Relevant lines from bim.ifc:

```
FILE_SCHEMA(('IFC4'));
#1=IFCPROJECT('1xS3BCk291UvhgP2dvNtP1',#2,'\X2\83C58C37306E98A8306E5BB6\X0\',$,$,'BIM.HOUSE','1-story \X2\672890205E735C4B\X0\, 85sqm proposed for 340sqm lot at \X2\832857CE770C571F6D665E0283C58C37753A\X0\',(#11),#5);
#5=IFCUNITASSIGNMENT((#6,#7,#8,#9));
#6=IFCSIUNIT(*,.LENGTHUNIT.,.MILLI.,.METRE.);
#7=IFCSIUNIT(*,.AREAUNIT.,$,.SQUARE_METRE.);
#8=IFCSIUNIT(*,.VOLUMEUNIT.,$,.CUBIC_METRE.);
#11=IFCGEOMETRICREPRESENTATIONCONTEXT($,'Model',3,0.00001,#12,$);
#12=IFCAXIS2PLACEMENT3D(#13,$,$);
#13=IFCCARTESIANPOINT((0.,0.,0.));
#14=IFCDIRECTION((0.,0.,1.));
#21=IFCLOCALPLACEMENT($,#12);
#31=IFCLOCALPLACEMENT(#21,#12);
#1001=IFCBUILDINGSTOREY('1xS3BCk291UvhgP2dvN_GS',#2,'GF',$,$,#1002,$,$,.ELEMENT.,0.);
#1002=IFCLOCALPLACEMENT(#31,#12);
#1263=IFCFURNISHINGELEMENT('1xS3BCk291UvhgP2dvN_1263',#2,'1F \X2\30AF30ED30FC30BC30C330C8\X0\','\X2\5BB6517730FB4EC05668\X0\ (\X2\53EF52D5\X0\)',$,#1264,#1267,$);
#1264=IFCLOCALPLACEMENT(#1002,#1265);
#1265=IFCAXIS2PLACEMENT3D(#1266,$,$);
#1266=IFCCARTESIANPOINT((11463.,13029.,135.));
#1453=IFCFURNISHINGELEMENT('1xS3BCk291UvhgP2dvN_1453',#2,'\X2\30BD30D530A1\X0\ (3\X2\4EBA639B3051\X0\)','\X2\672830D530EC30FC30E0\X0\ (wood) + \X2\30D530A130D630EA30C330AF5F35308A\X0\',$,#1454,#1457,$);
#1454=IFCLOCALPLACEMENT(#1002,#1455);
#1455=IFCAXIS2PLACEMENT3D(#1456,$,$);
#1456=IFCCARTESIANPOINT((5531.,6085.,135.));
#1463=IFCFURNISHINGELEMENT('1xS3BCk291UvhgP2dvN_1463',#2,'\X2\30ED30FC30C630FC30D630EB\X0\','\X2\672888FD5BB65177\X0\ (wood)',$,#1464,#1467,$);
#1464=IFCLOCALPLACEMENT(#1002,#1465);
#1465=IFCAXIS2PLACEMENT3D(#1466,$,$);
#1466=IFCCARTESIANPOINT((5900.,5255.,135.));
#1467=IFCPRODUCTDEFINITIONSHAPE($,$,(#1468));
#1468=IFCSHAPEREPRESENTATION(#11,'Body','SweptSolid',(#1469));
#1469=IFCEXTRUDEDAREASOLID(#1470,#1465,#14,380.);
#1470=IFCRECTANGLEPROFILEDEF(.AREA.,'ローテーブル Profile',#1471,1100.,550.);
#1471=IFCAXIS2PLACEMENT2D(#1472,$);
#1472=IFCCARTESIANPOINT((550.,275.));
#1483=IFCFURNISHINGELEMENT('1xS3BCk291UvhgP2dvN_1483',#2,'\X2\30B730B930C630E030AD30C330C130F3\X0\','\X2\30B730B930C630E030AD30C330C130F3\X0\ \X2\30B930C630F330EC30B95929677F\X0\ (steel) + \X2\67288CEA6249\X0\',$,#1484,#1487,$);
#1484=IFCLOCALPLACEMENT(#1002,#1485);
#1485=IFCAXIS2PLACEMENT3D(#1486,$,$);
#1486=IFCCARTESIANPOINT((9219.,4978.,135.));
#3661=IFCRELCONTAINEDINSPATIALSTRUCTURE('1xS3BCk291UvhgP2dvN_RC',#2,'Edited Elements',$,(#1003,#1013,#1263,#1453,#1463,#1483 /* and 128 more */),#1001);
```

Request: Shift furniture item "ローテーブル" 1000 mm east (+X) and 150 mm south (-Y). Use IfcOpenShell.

```python
import ifcopenshell
import ifcopenshell.api.geometry
import ifcopenshell.util.placement
import ifcopenshell.util.unit

model = ifcopenshell.open("bim.ifc")
unit_scale = ifcopenshell.util.unit.calculate_unit_scale(model)

item = model.by_id(1463)
matrix = ifcopenshell.util.placement.get_local_placement(item.ObjectPlacement)
matrix[0, 3] += 1 / unit_scale
matrix[1, 3] -= 0.15 / unit_scale
ifcopenshell.api.geometry.edit_object_placement(model, product=item, matrix=matrix, is_si=False)

print(ifcopenshell.util.placement.get_local_placement(item.ObjectPlacement).round(3) + 0.0)

model.write("bim-out.ifc")
```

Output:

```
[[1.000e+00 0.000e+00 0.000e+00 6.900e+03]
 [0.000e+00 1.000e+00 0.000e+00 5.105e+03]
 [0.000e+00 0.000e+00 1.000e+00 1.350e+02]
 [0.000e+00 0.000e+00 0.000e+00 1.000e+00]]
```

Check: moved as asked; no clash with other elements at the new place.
